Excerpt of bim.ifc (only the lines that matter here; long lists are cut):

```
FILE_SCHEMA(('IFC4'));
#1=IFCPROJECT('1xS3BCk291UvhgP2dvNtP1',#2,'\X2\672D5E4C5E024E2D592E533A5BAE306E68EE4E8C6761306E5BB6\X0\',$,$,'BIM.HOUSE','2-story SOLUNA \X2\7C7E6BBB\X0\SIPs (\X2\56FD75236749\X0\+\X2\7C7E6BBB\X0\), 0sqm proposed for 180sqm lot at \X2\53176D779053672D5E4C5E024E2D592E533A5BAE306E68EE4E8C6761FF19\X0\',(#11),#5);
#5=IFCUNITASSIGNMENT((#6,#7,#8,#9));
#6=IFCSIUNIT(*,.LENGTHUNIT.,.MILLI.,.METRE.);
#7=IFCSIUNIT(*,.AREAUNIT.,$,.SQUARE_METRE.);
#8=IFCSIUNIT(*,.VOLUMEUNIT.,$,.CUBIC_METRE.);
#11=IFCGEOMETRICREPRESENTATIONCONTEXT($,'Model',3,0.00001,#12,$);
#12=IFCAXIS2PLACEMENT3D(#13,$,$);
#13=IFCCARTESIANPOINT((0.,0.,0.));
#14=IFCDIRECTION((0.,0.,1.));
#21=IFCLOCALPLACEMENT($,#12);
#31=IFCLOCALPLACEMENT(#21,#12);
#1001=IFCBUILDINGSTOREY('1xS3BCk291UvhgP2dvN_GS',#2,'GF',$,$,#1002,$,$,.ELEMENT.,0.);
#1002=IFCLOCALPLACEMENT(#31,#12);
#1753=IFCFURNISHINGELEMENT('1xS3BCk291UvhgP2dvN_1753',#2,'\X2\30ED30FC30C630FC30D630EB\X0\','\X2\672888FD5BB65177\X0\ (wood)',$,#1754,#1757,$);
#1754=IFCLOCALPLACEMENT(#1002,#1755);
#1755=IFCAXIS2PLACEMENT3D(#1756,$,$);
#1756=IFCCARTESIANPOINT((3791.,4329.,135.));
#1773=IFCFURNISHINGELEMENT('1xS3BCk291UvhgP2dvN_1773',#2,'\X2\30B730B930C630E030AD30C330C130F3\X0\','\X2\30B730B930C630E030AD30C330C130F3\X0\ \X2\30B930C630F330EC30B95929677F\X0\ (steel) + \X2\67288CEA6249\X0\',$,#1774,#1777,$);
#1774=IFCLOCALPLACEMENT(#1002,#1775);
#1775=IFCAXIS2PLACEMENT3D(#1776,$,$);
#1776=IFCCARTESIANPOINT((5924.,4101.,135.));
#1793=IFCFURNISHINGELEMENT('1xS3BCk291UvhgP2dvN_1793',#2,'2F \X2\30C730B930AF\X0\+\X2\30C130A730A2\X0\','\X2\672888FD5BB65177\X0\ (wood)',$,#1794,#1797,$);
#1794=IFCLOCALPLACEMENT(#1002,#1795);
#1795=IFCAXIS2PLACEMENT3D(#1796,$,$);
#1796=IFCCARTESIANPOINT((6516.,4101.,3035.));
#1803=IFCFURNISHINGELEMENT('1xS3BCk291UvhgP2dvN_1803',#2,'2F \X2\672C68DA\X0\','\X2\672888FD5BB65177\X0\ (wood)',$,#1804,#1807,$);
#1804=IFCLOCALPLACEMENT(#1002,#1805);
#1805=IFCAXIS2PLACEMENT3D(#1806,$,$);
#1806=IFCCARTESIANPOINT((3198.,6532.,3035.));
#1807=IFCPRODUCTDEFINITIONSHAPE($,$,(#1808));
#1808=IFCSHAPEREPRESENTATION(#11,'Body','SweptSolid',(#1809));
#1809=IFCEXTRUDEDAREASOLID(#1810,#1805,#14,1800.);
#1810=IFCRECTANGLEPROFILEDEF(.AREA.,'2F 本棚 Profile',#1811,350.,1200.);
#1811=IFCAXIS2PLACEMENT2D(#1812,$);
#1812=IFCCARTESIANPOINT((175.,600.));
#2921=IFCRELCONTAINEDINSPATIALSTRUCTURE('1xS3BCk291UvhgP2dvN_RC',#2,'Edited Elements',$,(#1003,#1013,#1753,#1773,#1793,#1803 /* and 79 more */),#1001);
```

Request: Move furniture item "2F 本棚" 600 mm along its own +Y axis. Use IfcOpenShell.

```python
import ifcopenshell
import ifcopenshell.api.geometry
import ifcopenshell.util.placement
import ifcopenshell.util.unit

model = ifcopenshell.open("bim.ifc")
unit_scale = ifcopenshell.util.unit.calculate_unit_scale(model)

item = model.by_guid("1xS3BCk291UvhgP2dvN_1803")
matrix = ifcopenshell.util.placement.get_local_placement(item.ObjectPlacement)
matrix[:3, 3] += matrix[:3, 1] * 0.6 / unit_scale
ifcopenshell.api.geometry.edit_object_placement(model, product=item, matrix=matrix, is_si=False)

print(ifcopenshell.util.placement.get_local_placement(item.ObjectPlacement).round(3) + 0.0)

model.write("bim_rev.ifc")
```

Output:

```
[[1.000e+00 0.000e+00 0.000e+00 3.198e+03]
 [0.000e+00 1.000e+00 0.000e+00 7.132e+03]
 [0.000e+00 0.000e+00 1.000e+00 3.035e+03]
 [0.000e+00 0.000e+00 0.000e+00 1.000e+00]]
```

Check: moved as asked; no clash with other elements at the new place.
